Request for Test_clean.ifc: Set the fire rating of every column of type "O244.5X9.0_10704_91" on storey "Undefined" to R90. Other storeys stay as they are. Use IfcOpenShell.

First a look at what the model holds.

```python
import ifcopenshell
import ifcopenshell.util.element

model = ifcopenshell.open("Test_clean.ifc")
print(model.schema)
storey = next(s for s in model.by_type("IfcBuildingStorey") if s.Name == "Undefined")
columns = [e for e in ifcopenshell.util.element.get_decomposition(storey) if e.is_a("IfcColumn")]
seen = {}
for e in columns:
    element_type = ifcopenshell.util.element.get_type(e)
    key = (element_type.Name if element_type != e and element_type else None, ifcopenshell.util.element.get_pset(e, "Pset_ColumnCommon", "FireRating"))
    seen[key] = seen.get(key, 0) + 1
for (name, value), count in sorted(seen.items(), key=str):
    print(count, "x", name, "|", value)
```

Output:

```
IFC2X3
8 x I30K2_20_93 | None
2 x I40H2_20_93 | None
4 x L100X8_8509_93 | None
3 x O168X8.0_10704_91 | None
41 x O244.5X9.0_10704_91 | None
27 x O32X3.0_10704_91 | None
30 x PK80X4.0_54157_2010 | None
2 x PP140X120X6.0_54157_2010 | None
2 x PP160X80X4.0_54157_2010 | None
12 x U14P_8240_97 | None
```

```python
import ifcopenshell
import ifcopenshell.api.pset
import ifcopenshell.util.element

model = ifcopenshell.open("Test_clean.ifc")

storey = next(s for s in model.by_type("IfcBuildingStorey") if s.Name == "Undefined")
columns = [e for e in ifcopenshell.util.element.get_decomposition(storey) if e.is_a("IfcColumn")]

count = 0
for e in columns:
    element_type = ifcopenshell.util.element.get_type(e)
    if element_type in (None, e) or element_type.Name != "O244.5X9.0_10704_91":
        continue
    found = ifcopenshell.util.element.get_pset(e, "Pset_ColumnCommon", should_inherit=False)
    if found:
        pset = model.by_id(found["id"])
        if len(ifcopenshell.util.element.get_elements_by_pset(pset)) > 1:
            pset = ifcopenshell.api.pset.unshare_pset(model, products=[e], pset=pset)[0]
    else:
        pset = ifcopenshell.api.pset.add_pset(model, product=e, name="Pset_ColumnCommon")
    ifcopenshell.api.pset.edit_pset(model, pset=pset, properties={"FireRating": "R90"})
    count += 1

print(count, "columns updated")

model.write("Test_clean_v2.ifc")
```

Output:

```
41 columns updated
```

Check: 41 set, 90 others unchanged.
